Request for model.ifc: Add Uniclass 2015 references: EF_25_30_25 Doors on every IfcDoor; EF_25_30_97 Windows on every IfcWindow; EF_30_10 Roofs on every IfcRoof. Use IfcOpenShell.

First a look at what the model holds.

```python
import ifcopenshell

model = ifcopenshell.open("model.ifc")
print(model.schema)
print("classifications:", [c.Name for c in model.by_type("IfcClassification")])
for ifc_class in ("IfcDoor", "IfcRoof", "IfcStair", "IfcWall", "IfcWindow"):
    print(ifc_class, len(model.by_type(ifc_class)))
```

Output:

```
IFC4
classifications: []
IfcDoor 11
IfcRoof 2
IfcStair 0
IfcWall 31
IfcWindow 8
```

```python
import ifcopenshell
import ifcopenshell.api.classification

model = ifcopenshell.open("model.ifc")

system = ifcopenshell.api.classification.add_classification(model, classification="Uniclass 2015")

codes = {
    "IfcDoor": ("EF_25_30_25", "Doors"),
    "IfcWindow": ("EF_25_30_97", "Windows"),
    "IfcRoof": ("EF_30_10", "Roofs"),
}
for ifc_class, (code, name) in codes.items():
    products = model.by_type(ifc_class)
    ifcopenshell.api.classification.add_reference(
        model, products=products, classification=system, identification=code, name=name
    )
    print(code, len(products))

model.write("model_updated.ifc")
```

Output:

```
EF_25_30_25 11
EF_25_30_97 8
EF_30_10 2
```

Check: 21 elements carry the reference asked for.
